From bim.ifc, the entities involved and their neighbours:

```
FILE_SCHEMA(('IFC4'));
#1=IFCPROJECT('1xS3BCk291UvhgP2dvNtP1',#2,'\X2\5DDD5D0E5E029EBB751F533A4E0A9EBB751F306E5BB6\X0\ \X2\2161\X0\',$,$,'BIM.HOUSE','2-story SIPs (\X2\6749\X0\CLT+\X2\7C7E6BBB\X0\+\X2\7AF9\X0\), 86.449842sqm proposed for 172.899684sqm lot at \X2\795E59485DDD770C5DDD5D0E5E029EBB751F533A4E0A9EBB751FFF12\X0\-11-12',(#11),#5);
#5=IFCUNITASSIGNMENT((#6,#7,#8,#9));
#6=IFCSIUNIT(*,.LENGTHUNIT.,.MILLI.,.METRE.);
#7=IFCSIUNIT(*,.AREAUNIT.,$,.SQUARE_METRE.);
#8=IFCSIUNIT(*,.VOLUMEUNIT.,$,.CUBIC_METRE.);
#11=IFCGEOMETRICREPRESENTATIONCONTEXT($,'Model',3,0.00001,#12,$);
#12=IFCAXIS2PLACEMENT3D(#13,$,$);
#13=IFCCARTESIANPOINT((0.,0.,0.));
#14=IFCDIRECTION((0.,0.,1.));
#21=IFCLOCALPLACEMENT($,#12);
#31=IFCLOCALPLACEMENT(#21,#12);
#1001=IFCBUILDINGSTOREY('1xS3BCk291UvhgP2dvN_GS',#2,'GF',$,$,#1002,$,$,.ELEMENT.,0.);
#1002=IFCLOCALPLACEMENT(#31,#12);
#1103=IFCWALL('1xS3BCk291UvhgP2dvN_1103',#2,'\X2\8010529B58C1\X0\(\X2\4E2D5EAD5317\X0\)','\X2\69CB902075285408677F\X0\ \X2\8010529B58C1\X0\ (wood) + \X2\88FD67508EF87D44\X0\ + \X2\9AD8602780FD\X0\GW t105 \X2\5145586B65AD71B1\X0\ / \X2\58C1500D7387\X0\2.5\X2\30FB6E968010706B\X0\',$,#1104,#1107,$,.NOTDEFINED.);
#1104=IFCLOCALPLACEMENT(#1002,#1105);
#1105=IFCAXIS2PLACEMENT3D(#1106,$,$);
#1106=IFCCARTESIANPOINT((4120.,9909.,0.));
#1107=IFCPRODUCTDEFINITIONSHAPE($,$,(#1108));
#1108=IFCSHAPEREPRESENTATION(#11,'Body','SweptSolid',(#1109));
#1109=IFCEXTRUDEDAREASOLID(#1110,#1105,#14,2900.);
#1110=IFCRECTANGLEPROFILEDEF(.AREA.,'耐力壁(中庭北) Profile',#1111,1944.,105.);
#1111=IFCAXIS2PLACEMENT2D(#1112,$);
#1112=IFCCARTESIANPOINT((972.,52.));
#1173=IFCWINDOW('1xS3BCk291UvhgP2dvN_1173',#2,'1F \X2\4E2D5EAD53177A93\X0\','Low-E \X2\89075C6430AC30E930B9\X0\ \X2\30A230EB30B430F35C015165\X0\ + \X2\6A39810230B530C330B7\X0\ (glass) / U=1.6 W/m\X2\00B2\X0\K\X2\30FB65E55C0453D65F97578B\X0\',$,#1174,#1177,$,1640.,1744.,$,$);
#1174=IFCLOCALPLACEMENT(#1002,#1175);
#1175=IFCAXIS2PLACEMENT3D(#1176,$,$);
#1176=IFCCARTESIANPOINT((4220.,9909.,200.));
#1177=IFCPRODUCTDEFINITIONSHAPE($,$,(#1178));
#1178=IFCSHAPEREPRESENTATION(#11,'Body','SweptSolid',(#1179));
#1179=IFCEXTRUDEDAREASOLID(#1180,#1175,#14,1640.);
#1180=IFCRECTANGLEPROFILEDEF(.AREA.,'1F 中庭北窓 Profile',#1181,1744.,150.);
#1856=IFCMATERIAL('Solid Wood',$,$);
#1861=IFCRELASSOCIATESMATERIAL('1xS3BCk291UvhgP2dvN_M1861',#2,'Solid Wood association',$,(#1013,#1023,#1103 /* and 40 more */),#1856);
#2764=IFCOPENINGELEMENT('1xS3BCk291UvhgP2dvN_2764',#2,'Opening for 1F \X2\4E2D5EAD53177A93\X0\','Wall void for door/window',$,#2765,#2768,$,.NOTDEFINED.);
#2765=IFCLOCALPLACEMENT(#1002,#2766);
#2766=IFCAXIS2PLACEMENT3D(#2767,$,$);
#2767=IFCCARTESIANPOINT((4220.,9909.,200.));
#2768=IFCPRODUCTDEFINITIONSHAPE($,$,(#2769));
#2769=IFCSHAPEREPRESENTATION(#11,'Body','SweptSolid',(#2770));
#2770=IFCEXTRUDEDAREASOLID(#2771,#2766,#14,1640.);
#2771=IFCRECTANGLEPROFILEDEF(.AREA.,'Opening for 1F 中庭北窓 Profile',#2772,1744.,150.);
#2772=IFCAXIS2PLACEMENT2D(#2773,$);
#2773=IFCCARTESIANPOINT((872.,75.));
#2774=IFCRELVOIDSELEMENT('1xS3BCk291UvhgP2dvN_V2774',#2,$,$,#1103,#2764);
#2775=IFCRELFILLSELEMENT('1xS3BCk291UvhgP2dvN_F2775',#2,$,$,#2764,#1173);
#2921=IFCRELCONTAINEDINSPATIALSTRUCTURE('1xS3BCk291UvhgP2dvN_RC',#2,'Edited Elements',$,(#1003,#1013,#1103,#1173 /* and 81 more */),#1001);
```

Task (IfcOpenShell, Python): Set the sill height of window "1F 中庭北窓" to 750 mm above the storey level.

```python
import numpy as np
import ifcopenshell
import ifcopenshell.api.geometry
import ifcopenshell.geom
import ifcopenshell.util.element
import ifcopenshell.util.placement
import ifcopenshell.util.shape
import ifcopenshell.util.unit

model = ifcopenshell.open("bim.ifc")
unit_scale = ifcopenshell.util.unit.calculate_unit_scale(model)

window = model.by_guid("1xS3BCk291UvhgP2dvN_1173")
opening = window.FillsVoids[0].RelatingOpeningElement
storey = ifcopenshell.util.element.get_container(window, ifc_class="IfcBuildingStorey")
level = ifcopenshell.util.placement.get_local_placement(storey.ObjectPlacement)[2, 3]

# The opening's origin need not be at the sill, so measure its lowest point.
shape = ifcopenshell.geom.create_shape(ifcopenshell.geom.settings(), opening)
bottom = ifcopenshell.util.shape.get_shape_bottom_elevation(shape, shape.geometry) / unit_scale
dz = level + 0.75 / unit_scale - bottom

shift = np.array([0.0, 0.0, dz])
# The window is not placed relative to its opening, so move both.
for product in (opening, window):
    matrix = ifcopenshell.util.placement.get_local_placement(product.ObjectPlacement)
    matrix[:3, 3] += shift
    ifcopenshell.api.geometry.edit_object_placement(model, product=product, matrix=matrix, is_si=False)

print(f"moved by {dz * unit_scale:+.3f} m")

model.write("bim_v2.ifc")
```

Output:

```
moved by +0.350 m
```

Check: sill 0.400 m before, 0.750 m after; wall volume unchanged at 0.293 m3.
